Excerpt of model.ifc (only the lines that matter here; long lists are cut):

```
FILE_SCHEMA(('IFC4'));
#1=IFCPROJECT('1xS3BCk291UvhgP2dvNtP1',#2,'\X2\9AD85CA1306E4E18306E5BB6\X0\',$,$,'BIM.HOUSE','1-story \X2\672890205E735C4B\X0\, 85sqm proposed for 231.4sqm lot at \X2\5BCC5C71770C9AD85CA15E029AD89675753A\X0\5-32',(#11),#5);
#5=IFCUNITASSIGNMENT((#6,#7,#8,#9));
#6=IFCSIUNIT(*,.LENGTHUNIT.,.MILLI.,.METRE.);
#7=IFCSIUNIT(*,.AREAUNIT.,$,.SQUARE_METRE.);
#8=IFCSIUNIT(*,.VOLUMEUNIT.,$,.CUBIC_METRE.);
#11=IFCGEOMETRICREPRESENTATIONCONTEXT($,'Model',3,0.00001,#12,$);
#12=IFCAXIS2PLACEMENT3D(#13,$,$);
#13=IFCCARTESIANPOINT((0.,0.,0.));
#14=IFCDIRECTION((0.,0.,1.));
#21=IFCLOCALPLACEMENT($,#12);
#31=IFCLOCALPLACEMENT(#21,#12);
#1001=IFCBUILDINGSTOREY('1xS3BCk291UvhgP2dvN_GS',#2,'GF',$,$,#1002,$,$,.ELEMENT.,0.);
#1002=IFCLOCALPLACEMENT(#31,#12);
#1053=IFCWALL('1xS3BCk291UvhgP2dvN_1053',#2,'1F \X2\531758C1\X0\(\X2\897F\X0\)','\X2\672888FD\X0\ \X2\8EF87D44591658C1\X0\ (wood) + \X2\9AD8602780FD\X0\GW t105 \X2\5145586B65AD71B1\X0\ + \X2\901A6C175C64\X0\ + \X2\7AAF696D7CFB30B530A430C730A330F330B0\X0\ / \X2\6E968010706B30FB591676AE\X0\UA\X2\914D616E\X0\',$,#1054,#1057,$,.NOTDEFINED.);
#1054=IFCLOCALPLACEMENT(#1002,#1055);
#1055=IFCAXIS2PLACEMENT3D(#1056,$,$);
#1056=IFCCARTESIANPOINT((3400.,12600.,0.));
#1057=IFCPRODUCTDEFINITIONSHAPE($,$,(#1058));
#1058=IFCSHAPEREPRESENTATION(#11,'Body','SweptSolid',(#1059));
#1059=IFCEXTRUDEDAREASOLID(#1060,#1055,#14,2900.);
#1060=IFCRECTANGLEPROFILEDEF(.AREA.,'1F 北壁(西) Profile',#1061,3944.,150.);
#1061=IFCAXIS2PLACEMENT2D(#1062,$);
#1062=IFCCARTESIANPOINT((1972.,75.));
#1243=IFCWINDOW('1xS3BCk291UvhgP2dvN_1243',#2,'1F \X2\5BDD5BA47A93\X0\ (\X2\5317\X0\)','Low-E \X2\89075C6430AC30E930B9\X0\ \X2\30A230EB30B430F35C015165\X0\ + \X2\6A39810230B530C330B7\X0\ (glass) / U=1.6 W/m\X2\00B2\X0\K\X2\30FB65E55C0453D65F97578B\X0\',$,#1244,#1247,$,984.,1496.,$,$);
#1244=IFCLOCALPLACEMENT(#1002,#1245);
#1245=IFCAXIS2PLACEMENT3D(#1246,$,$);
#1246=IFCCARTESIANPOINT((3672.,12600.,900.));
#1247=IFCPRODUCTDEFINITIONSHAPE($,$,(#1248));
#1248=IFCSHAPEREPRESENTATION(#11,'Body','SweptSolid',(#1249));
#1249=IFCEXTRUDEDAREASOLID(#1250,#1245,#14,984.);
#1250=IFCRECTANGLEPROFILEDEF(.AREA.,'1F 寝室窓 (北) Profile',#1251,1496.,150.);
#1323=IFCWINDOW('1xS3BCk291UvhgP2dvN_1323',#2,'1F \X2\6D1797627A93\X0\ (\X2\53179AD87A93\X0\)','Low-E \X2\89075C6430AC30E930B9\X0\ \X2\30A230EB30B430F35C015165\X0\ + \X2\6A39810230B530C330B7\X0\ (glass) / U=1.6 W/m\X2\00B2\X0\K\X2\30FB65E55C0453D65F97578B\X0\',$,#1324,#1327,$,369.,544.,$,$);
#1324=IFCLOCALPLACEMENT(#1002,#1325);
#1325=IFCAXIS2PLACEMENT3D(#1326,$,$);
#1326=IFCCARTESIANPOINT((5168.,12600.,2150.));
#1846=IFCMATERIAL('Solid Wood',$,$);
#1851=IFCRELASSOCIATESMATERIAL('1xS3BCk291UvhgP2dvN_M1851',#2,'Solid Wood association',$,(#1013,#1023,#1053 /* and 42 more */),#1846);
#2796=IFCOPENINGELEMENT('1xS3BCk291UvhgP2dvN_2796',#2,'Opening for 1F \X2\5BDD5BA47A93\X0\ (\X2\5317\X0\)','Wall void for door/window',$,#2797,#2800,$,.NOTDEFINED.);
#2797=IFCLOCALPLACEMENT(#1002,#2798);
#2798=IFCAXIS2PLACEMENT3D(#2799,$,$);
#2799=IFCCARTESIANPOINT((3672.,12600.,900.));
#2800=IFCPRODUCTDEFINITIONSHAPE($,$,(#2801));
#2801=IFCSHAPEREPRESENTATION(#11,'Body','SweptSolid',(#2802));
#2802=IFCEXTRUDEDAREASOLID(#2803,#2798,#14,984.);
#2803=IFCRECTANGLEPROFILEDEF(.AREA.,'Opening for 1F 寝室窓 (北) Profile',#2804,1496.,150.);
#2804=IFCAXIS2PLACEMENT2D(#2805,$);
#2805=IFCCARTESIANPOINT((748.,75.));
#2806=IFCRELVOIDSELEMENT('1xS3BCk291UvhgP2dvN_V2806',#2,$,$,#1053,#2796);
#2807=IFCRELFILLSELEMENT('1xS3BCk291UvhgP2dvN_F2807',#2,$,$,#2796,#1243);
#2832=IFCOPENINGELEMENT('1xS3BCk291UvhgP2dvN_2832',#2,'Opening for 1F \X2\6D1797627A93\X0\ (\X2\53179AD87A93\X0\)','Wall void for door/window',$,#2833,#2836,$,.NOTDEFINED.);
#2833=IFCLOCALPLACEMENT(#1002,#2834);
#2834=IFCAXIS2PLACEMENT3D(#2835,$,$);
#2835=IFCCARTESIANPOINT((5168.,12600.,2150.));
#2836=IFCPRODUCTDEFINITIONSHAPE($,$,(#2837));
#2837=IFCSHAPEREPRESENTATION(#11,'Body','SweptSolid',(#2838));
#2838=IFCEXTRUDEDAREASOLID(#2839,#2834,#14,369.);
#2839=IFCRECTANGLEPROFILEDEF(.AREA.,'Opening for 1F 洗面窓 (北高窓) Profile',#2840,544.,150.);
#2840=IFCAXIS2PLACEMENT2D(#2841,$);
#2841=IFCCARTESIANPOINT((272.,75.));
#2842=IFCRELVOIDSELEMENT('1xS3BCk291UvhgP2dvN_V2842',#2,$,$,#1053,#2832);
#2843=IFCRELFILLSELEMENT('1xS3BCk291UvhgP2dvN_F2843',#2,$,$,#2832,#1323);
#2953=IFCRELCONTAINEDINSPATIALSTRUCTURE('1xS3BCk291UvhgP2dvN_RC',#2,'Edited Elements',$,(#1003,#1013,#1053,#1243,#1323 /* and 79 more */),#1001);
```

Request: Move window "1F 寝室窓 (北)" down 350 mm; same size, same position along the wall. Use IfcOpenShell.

```python
import numpy as np
import ifcopenshell
import ifcopenshell.api.geometry
import ifcopenshell.util.placement
import ifcopenshell.util.unit

model = ifcopenshell.open("model.ifc")
unit_scale = ifcopenshell.util.unit.calculate_unit_scale(model)

window = model.by_guid("1xS3BCk291UvhgP2dvN_1243")
opening = window.FillsVoids[0].RelatingOpeningElement
dz = -350.0

shift = np.array([0.0, 0.0, dz])
# The window is not placed relative to its opening, so move both.
for product in (opening, window):
    matrix = ifcopenshell.util.placement.get_local_placement(product.ObjectPlacement)
    matrix[:3, 3] += shift
    ifcopenshell.api.geometry.edit_object_placement(model, product=product, matrix=matrix, is_si=False)

print(f"moved by {dz * unit_scale:+.3f} m")

model.write("model_updated.ifc")
```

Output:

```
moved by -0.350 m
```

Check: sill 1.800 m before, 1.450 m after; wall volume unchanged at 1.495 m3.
